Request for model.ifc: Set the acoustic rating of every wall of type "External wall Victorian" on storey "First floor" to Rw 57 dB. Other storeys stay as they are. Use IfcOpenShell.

First a look at what the model holds.

```python
import ifcopenshell
import ifcopenshell.util.element

model = ifcopenshell.open("model.ifc")
print(model.schema)
storey = next(s for s in model.by_type("IfcBuildingStorey") if s.Name == "First floor")
walls = [e for e in ifcopenshell.util.element.get_decomposition(storey) if e.is_a("IfcWall")]
seen = {}
for e in walls:
    element_type = ifcopenshell.util.element.get_type(e)
    key = (element_type.Name if element_type != e and element_type else None, ifcopenshell.util.element.get_pset(e, "Pset_WallCommon", "AcousticRating"))
    seen[key] = seen.get(key, 0) + 1
for (name, value), count in sorted(seen.items(), key=str):
    print(count, "x", name, "|", value)
```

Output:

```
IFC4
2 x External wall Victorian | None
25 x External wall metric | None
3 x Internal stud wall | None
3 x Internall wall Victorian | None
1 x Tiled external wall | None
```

```python
import ifcopenshell
import ifcopenshell.api.pset
import ifcopenshell.util.element

model = ifcopenshell.open("model.ifc")

storey = next(s for s in model.by_type("IfcBuildingStorey") if s.Name == "First floor")
walls = [e for e in ifcopenshell.util.element.get_decomposition(storey) if e.is_a("IfcWall")]

count = 0
for e in walls:
    element_type = ifcopenshell.util.element.get_type(e)
    if element_type in (None, e) or element_type.Name != "External wall Victorian":
        continue
    # add_pset returns the element's existing set when there is one.
    pset = ifcopenshell.api.pset.add_pset(model, product=e, name="Pset_WallCommon")
    ifcopenshell.api.pset.edit_pset(model, pset=pset, properties={"AcousticRating": "Rw 57 dB"})
    count += 1

print(count, "walls updated")

model.write("model_rev.ifc")
```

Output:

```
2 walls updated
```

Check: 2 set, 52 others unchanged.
